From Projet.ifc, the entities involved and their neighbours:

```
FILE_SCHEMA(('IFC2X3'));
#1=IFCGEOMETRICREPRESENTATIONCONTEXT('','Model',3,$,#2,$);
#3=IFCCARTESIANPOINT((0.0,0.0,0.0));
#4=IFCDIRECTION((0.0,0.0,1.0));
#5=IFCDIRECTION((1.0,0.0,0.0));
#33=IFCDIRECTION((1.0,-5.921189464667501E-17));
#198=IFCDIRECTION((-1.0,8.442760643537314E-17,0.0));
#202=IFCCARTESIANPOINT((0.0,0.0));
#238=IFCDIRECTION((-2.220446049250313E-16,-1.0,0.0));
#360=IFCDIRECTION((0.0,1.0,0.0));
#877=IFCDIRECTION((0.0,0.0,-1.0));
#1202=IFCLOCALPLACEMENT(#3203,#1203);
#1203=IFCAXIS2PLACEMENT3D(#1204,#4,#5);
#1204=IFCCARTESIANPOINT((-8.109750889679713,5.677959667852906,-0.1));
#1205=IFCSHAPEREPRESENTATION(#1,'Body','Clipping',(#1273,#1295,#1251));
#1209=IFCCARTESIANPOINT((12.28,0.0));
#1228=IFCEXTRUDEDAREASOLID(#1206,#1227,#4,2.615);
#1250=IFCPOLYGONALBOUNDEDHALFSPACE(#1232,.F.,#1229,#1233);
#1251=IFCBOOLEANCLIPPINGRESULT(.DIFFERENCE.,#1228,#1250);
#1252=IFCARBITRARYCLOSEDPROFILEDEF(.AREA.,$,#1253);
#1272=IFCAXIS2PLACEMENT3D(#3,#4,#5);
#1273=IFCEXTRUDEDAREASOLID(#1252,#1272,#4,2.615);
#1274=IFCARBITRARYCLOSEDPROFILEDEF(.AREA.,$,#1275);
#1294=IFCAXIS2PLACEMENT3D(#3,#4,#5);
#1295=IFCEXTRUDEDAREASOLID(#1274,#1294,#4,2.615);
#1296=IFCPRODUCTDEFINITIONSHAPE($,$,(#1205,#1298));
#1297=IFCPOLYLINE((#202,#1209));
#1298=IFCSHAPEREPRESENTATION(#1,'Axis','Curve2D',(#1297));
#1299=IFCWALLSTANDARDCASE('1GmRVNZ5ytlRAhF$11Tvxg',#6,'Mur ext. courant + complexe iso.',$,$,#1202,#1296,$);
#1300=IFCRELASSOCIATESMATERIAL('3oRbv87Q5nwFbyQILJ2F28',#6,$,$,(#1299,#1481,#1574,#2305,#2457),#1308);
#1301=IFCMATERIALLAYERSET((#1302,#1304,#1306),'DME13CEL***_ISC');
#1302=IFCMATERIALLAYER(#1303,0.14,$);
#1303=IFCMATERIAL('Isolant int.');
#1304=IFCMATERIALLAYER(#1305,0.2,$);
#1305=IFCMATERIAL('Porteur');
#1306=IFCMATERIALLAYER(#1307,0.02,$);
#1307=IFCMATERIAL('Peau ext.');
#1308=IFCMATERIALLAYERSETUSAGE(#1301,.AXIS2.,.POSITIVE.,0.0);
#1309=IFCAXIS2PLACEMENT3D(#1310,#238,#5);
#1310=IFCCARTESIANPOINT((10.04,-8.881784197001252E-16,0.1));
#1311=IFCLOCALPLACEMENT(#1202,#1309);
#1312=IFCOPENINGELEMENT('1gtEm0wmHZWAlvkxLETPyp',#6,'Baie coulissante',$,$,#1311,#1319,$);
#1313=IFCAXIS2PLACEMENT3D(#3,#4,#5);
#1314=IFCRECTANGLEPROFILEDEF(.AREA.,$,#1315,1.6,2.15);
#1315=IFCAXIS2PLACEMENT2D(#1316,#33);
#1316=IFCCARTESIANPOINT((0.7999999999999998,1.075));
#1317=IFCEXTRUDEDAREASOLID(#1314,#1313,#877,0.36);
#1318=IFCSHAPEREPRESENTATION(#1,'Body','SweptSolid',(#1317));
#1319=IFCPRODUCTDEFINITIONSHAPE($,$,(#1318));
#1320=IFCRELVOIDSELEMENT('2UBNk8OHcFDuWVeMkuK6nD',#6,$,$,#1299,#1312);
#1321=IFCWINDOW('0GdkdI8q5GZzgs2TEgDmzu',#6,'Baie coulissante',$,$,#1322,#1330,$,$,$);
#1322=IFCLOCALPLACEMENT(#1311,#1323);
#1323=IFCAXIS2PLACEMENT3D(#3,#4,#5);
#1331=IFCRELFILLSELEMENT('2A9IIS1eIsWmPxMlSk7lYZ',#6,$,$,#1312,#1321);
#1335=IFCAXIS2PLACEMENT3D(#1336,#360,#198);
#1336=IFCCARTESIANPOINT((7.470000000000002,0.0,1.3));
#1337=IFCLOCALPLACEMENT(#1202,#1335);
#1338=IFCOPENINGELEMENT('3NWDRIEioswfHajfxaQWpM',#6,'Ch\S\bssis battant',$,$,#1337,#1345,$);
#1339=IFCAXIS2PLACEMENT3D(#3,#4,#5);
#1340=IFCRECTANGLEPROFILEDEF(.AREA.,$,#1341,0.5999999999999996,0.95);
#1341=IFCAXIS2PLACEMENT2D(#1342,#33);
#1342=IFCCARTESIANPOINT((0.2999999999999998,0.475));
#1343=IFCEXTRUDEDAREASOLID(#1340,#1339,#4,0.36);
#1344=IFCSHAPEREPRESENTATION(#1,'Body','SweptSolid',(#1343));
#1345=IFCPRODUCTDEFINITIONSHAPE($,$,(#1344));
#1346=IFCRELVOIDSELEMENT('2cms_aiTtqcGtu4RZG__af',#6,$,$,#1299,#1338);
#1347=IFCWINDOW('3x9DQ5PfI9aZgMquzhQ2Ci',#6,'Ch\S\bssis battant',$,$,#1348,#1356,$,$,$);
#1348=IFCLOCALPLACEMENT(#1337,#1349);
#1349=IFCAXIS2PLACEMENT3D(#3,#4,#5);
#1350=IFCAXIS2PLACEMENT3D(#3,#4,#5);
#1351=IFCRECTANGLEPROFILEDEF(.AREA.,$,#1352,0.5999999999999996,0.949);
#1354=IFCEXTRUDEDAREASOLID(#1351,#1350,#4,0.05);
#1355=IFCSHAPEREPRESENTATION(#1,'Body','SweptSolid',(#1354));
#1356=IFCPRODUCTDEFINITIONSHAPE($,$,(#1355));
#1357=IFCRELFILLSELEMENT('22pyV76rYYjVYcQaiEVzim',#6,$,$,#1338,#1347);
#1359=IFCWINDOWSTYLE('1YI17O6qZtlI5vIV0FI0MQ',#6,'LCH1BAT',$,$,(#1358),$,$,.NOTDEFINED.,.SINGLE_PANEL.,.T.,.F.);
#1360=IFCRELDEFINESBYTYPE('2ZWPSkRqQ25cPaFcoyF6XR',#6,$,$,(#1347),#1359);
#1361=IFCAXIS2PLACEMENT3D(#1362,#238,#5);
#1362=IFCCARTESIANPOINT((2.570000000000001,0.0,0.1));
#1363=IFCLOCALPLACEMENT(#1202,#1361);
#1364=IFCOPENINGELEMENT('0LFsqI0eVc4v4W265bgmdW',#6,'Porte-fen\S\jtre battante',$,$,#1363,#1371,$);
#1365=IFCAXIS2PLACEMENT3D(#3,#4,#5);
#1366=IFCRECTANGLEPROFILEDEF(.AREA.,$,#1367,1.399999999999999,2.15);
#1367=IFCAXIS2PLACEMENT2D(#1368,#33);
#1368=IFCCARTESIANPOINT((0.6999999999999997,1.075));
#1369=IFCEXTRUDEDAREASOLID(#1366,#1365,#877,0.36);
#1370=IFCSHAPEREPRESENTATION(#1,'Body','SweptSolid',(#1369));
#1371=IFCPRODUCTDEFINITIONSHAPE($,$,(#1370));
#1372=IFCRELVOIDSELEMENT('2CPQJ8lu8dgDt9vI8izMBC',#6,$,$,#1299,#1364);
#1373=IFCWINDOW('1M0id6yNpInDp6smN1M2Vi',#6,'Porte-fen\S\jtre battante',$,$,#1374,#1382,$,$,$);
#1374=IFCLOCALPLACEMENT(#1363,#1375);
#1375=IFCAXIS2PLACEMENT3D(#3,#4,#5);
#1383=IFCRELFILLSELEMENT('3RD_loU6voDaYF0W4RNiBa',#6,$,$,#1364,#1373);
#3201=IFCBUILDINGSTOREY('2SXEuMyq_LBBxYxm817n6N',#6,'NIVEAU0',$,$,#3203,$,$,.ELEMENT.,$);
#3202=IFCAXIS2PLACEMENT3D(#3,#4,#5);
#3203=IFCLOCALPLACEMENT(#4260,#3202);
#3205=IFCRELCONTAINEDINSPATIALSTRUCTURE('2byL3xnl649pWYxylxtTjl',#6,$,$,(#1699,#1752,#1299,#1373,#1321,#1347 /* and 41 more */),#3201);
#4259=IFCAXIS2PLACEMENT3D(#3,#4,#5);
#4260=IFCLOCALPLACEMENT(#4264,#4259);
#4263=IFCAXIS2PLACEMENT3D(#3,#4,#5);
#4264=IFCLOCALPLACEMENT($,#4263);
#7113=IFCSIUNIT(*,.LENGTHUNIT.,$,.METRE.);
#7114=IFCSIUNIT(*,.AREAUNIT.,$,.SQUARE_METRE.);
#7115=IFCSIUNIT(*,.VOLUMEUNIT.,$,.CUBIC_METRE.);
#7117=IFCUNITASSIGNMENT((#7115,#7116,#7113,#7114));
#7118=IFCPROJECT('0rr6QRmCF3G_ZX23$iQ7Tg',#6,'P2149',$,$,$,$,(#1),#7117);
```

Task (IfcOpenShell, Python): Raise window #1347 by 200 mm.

```python
import numpy as np
import ifcopenshell
import ifcopenshell.api.geometry
import ifcopenshell.util.placement
import ifcopenshell.util.unit

model = ifcopenshell.open("Projet.ifc")
unit_scale = ifcopenshell.util.unit.calculate_unit_scale(model)

window = model.by_guid("3x9DQ5PfI9aZgMquzhQ2Ci")
opening = window.FillsVoids[0].RelatingOpeningElement
dz = 0.2 / unit_scale

shift = np.array([0.0, 0.0, dz])
# The window is placed relative to its opening, so it follows when the opening moves.
matrix = ifcopenshell.util.placement.get_local_placement(opening.ObjectPlacement)
matrix[:3, 3] += shift
ifcopenshell.api.geometry.edit_object_placement(
    model, product=opening, matrix=matrix, is_si=False, should_transform_children=True
)

print(f"moved by {dz * unit_scale:+.3f} m")

model.write("Projet_v2.ifc")
```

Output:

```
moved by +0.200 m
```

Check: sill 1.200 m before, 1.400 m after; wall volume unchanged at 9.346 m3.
